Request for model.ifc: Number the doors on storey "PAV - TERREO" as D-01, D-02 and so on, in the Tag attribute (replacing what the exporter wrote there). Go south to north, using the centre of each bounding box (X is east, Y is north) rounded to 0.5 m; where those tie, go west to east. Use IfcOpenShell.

First a look at what the model holds.

```python
import ifcopenshell
import ifcopenshell.util.element
import ifcopenshell.util.placement

model = ifcopenshell.open("model.ifc")
print(model.schema)
storey = next(s for s in model.by_type("IfcBuildingStorey") if s.Name == "PAV - TERREO")
doors = [e for e in ifcopenshell.util.element.get_decomposition(storey) if e.is_a("IfcDoor")]
for e in sorted(doors, key=lambda e: e.id()):
    origin = ifcopenshell.util.placement.get_local_placement(e.ObjectPlacement)[:3, 3]
    print(e.id(), e.Tag, e.Name, origin.round(2) + 0.0, sep=" | ")
```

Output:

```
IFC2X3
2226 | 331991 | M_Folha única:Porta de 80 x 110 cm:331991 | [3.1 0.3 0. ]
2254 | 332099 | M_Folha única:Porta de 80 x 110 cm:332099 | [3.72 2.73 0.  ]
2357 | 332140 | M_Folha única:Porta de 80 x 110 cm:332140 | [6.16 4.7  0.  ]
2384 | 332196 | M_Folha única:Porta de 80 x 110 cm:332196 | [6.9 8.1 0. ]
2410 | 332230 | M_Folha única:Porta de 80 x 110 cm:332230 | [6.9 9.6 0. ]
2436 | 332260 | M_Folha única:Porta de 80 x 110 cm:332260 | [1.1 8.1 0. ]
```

```python
import ifcopenshell
import ifcopenshell.geom
import ifcopenshell.util.element
import ifcopenshell.util.shape

model = ifcopenshell.open("model.ifc")
settings = ifcopenshell.geom.settings()
settings.set("use-world-coords", True)


def centre(element):
    shape = ifcopenshell.geom.create_shape(settings, element)
    return ifcopenshell.util.shape.get_bbox_centroid(shape.geometry)


storey = next(s for s in model.by_type("IfcBuildingStorey") if s.Name == "PAV - TERREO")
doors = [e for e in ifcopenshell.util.element.get_decomposition(storey) if e.is_a("IfcDoor")]

# Insertion points can sit at a corner or the storey origin, so sort by the geometry (in metres).
centres = {e: centre(e) for e in doors}
doors.sort(key=lambda e: (round(centres[e][1] / 0.5), centres[e][0]))

for i, e in enumerate(doors, start=1):
    number = f"D-{i:02d}"
    e.Tag = number
    print(e.id(), number)

model.write("model_edited.ifc")
```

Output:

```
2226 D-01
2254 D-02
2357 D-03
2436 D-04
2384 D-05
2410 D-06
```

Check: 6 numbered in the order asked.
